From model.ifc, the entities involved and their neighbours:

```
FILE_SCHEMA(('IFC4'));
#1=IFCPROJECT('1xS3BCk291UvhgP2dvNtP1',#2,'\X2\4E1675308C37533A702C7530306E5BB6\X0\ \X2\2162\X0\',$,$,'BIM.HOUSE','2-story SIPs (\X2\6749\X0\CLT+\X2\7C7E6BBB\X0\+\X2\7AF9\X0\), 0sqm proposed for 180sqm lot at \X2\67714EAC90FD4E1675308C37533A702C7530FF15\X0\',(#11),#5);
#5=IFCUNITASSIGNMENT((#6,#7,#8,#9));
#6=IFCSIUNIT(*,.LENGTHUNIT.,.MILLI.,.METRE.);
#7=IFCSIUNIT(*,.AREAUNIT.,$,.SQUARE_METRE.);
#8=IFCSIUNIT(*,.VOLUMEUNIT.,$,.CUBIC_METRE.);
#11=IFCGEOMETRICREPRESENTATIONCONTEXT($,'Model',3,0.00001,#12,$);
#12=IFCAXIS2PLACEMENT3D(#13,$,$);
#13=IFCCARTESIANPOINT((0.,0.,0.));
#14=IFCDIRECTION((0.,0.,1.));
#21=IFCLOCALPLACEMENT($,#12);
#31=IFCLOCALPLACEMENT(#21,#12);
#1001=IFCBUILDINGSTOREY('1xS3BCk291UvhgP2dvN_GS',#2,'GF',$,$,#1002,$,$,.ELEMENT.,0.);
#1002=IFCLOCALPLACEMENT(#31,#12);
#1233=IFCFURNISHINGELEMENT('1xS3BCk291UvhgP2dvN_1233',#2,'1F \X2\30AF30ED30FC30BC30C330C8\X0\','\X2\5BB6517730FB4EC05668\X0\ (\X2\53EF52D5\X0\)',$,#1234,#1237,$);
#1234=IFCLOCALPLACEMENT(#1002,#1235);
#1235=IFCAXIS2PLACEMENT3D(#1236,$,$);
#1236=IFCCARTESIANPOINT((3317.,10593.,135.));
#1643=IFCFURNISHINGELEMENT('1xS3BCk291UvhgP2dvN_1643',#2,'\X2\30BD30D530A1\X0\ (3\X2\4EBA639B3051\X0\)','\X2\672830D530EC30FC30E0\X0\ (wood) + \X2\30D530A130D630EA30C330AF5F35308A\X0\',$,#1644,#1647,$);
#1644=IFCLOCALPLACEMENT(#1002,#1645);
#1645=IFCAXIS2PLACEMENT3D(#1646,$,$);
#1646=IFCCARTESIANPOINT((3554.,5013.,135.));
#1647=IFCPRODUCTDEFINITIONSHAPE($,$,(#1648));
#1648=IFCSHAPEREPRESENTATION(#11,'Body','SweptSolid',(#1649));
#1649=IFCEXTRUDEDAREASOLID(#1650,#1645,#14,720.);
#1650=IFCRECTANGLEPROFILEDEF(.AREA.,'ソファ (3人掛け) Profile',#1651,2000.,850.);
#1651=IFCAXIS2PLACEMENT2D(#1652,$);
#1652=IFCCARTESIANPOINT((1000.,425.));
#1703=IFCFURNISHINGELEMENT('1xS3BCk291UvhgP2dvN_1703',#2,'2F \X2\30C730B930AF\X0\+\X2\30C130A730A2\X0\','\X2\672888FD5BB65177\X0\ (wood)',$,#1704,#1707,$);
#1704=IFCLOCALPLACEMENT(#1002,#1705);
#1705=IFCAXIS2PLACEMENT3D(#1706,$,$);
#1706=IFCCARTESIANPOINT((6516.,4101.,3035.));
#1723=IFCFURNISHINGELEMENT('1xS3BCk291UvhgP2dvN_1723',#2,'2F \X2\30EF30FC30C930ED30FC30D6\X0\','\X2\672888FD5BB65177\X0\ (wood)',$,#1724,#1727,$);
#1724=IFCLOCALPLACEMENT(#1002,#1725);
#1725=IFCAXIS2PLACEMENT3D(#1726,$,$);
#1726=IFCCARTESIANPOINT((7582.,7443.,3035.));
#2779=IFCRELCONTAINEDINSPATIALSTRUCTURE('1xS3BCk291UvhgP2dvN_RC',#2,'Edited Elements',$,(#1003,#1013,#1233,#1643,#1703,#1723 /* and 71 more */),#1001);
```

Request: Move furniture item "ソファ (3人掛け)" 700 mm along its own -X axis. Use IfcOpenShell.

```python
import ifcopenshell
import ifcopenshell.api.geometry
import ifcopenshell.util.placement

model = ifcopenshell.open("model.ifc")

item = model.by_id(1643)
matrix = ifcopenshell.util.placement.get_local_placement(item.ObjectPlacement)
matrix[:3, 3] -= matrix[:3, 0] * 700.0
ifcopenshell.api.geometry.edit_object_placement(model, product=item, matrix=matrix, is_si=False)

print(ifcopenshell.util.placement.get_local_placement(item.ObjectPlacement).round(3) + 0.0)

model.write("model_edited.ifc")
```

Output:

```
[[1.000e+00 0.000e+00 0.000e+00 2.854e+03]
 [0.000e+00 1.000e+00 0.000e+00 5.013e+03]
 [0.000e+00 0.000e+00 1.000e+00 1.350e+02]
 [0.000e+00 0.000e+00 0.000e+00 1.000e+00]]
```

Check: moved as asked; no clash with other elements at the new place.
